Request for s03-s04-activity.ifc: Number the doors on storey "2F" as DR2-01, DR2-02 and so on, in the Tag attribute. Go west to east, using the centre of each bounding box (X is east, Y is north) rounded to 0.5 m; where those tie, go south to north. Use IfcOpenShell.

First a look at what the model holds.

```python
import ifcopenshell
import ifcopenshell.util.element
import ifcopenshell.util.placement

model = ifcopenshell.open("s03-s04-activity.ifc")
print(model.schema)
storey = next(s for s in model.by_type("IfcBuildingStorey") if s.Name == "2F")
doors = [e for e in ifcopenshell.util.element.get_decomposition(storey) if e.is_a("IfcDoor")]
for e in sorted(doors, key=lambda e: e.id()):
    origin = ifcopenshell.util.placement.get_local_placement(e.ObjectPlacement)[:3, 3]
    print(e.id(), e.Tag, e.Name, origin.round(2) + 0.0, sep=" | ")
```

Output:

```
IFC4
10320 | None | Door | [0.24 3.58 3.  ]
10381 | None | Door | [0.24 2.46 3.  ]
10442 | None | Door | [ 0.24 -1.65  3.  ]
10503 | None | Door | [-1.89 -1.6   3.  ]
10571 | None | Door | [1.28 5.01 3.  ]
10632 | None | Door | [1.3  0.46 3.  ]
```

```python
import ifcopenshell
import ifcopenshell.geom
import ifcopenshell.util.element
import ifcopenshell.util.shape

model = ifcopenshell.open("s03-s04-activity.ifc")
settings = ifcopenshell.geom.settings()
settings.set("use-world-coords", True)


def centre(element):
    shape = ifcopenshell.geom.create_shape(settings, element)
    return ifcopenshell.util.shape.get_bbox_centroid(shape.geometry)


storey = next(s for s in model.by_type("IfcBuildingStorey") if s.Name == "2F")
doors = [e for e in ifcopenshell.util.element.get_decomposition(storey) if e.is_a("IfcDoor")]

# Insertion points can sit at a corner or the storey origin, so sort by the geometry (in metres).
centres = {e: centre(e) for e in doors}
doors.sort(key=lambda e: (round(centres[e][0] / 0.5), centres[e][1]))

for i, e in enumerate(doors, start=1):
    number = f"DR2-{i:02d}"
    e.Tag = number
    print(e.id(), number)

model.write("s03-s04-activity_v2.ifc")
```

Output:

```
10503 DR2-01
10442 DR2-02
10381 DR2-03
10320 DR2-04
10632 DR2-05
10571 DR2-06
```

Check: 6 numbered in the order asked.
